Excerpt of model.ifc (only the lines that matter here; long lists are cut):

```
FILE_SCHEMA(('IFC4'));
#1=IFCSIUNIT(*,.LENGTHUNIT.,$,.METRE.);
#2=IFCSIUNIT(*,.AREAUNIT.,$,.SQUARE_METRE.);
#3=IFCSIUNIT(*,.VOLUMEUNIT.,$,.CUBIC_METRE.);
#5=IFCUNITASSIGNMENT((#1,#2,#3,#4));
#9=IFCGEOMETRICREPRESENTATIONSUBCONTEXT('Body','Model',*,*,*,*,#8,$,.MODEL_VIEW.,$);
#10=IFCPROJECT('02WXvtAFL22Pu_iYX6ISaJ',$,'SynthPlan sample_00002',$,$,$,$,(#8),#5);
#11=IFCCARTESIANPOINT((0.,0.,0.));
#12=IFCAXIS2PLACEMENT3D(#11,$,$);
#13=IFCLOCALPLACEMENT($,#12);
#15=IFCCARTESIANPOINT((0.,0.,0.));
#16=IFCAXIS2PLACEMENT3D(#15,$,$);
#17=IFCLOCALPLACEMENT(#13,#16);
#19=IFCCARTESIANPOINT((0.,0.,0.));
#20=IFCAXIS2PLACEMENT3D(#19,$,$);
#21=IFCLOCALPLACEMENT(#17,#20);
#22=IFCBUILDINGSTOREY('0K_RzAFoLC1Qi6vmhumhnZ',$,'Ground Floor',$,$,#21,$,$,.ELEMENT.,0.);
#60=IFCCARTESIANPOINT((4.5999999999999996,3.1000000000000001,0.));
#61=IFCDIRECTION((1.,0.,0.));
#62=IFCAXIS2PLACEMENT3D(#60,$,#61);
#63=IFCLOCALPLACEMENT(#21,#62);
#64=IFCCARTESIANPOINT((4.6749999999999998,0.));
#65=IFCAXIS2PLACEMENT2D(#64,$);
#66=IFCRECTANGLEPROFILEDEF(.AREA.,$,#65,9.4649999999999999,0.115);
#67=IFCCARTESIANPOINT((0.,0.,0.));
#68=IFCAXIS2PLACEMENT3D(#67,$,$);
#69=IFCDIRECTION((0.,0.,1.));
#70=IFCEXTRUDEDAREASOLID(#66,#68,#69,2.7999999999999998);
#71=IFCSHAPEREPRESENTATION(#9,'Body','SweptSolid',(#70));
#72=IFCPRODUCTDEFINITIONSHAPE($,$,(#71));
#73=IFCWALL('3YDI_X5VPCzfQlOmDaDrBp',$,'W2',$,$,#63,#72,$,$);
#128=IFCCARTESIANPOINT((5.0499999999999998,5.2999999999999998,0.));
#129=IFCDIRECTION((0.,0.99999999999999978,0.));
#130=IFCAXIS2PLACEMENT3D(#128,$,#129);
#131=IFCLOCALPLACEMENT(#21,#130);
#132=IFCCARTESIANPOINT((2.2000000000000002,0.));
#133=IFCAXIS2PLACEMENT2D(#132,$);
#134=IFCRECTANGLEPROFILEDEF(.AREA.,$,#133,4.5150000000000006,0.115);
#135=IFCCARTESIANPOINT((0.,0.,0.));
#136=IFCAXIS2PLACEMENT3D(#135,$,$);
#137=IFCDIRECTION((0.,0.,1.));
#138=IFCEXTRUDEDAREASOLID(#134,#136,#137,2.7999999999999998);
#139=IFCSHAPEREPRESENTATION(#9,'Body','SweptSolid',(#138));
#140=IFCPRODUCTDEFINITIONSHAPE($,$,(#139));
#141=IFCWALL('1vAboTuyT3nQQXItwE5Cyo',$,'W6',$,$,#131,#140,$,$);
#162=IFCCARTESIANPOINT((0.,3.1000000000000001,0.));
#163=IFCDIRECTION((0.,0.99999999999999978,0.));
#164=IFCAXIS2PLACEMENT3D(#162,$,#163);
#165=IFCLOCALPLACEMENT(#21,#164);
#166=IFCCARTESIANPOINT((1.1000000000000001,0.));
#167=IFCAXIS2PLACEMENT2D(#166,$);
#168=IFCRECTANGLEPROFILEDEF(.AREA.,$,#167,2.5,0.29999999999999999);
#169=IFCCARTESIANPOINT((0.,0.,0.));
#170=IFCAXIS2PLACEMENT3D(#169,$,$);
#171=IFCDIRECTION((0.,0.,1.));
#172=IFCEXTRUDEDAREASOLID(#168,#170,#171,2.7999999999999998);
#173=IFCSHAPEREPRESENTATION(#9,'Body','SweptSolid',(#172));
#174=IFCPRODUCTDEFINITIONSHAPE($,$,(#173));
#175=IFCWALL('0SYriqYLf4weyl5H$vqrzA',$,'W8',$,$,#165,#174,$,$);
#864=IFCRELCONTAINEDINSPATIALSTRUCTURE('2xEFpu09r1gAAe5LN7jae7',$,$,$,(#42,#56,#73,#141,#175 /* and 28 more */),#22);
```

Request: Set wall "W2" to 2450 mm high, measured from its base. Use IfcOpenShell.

```python
import ifcopenshell
import ifcopenshell.geom
import ifcopenshell.util.representation
import ifcopenshell.util.shape
import ifcopenshell.util.unit

model = ifcopenshell.open("model.ifc")
unit_scale = ifcopenshell.util.unit.calculate_unit_scale(model)
settings = ifcopenshell.geom.settings()


def volume(element):
    """Net volume in cubic metres, openings subtracted."""
    shape = ifcopenshell.geom.create_shape(settings, element)
    return ifcopenshell.util.shape.get_volume(shape.geometry)


wall = model.by_guid("3YDI_X5VPCzfQlOmDaDrBp")
before = volume(wall)

body = ifcopenshell.util.representation.get_representation(wall, "Model", "Body")
solid = body.Items[0]
old_height = solid.Depth
solid.Depth = 2.45 / unit_scale
after = volume(wall)

print(f"height {old_height:g} -> {solid.Depth:g}, volume {before:.3f} -> {after:.3f} m3")

model.write("model_v2.ifc")
```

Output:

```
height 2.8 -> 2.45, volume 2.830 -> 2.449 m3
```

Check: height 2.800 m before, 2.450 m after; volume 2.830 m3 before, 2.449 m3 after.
